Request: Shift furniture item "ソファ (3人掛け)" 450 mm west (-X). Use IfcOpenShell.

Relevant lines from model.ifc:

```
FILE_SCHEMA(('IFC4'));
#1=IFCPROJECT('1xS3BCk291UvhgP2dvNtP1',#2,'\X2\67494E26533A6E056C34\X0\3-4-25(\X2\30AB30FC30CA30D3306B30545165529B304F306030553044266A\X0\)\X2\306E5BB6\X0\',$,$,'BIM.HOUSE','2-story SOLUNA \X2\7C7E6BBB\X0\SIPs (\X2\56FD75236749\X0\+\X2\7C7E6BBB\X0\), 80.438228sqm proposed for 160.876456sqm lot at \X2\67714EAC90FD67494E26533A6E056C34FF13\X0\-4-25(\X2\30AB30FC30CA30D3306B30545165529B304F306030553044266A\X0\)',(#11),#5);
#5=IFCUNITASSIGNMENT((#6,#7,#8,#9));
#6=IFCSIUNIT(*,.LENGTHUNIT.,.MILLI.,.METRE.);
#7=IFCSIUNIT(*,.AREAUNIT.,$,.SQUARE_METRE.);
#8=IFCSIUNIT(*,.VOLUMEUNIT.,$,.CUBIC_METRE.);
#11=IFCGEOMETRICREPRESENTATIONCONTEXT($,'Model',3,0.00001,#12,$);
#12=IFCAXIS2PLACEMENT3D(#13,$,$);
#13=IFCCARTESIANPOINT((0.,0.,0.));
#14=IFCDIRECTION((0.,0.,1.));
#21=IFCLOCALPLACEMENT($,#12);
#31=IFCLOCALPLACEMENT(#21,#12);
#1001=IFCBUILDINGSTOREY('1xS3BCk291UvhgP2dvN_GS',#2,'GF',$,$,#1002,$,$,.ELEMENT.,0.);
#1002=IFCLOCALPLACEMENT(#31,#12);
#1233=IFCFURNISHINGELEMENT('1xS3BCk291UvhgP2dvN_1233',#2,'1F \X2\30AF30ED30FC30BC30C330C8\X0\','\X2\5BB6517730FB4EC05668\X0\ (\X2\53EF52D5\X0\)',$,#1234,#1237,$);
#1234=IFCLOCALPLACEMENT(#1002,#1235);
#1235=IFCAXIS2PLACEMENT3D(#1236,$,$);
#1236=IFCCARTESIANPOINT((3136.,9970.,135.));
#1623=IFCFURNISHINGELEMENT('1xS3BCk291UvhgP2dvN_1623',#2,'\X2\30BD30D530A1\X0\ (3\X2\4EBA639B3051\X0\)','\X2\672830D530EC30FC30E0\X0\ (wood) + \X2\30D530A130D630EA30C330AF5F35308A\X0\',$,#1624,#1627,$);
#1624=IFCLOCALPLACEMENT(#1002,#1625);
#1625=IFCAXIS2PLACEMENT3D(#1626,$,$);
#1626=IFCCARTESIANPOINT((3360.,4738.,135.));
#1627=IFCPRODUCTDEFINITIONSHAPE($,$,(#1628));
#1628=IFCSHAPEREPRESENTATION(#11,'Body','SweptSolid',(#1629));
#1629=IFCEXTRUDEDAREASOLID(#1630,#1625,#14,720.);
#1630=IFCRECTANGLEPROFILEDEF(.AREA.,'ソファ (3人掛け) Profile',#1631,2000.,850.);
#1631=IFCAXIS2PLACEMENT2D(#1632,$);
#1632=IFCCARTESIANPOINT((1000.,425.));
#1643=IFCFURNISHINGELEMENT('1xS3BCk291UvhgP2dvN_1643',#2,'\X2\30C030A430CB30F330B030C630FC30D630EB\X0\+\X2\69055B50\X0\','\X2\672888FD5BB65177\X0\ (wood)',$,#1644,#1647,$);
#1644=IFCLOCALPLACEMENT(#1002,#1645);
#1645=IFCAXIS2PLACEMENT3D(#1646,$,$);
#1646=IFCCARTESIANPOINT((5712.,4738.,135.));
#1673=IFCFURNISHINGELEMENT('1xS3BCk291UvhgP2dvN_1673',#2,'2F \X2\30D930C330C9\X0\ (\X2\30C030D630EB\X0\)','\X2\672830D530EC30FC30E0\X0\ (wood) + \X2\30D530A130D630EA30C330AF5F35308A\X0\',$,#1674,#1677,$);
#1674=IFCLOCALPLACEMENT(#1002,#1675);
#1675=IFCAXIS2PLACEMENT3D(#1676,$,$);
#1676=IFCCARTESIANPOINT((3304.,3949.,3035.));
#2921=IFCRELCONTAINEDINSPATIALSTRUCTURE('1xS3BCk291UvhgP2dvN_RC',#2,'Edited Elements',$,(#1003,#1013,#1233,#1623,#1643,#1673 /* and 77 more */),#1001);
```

```python
import ifcopenshell
import ifcopenshell.api.geometry
import ifcopenshell.util.placement
import ifcopenshell.util.unit

model = ifcopenshell.open("model.ifc")
unit_scale = ifcopenshell.util.unit.calculate_unit_scale(model)

item = model.by_guid("1xS3BCk291UvhgP2dvN_1623")
matrix = ifcopenshell.util.placement.get_local_placement(item.ObjectPlacement)
matrix[0, 3] -= 0.45 / unit_scale
ifcopenshell.api.geometry.edit_object_placement(model, product=item, matrix=matrix, is_si=False)

print(ifcopenshell.util.placement.get_local_placement(item.ObjectPlacement).round(3) + 0.0)

model.write("model_updated.ifc")
```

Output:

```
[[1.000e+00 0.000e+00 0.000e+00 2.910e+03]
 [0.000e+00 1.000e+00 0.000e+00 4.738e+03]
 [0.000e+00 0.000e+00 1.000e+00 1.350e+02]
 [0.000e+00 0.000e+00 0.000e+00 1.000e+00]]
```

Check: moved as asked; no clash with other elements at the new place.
